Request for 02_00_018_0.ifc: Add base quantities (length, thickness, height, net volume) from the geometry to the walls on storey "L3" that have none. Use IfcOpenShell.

First a look at what the model holds.

```python
import ifcopenshell
import ifcopenshell.util.element
import ifcopenshell.util.unit

model = ifcopenshell.open("02_00_018_0.ifc")
print(model.schema)
for unit_type in ("LENGTHUNIT", "AREAUNIT", "VOLUMEUNIT"):
    print(unit_type, ifcopenshell.util.unit.calculate_unit_scale(model, unit_type))
storey = next(s for s in model.by_type("IfcBuildingStorey") if s.Name == "L3")
walls = [e for e in ifcopenshell.util.element.get_decomposition(storey) if e.is_a("IfcWall")]
for e in sorted(walls, key=lambda e: e.id()):
    print(e.id(), e.is_a(), e.Name, list(ifcopenshell.util.element.get_psets(e, qtos_only=True)), sep=" | ")
```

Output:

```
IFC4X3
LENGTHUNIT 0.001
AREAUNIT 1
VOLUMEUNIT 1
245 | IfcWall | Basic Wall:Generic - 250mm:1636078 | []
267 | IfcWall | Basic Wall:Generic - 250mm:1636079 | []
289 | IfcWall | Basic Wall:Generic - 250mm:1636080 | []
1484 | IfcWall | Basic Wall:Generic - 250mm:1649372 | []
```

```python
import ifcopenshell
import ifcopenshell.api.pset
import ifcopenshell.geom
import ifcopenshell.util.element
import ifcopenshell.util.shape
import ifcopenshell.util.unit

model = ifcopenshell.open("02_00_018_0.ifc")
unit_scale = ifcopenshell.util.unit.calculate_unit_scale(model)
volume_scale = ifcopenshell.util.unit.calculate_unit_scale(model, "VOLUMEUNIT")
settings = ifcopenshell.geom.settings()

storey = next(s for s in model.by_type("IfcBuildingStorey") if s.Name == "L3")
walls = [e for e in ifcopenshell.util.element.get_decomposition(storey) if e.is_a("IfcWall")]

for e in sorted(walls, key=lambda e: e.id()):
    if ifcopenshell.util.element.get_psets(e, qtos_only=True, should_inherit=False):
        continue
    # Geometry comes back in metres, in the element's own axes.
    shape = ifcopenshell.geom.create_shape(settings, e)
    values = {
        "Length": ifcopenshell.util.shape.get_x(shape.geometry) / unit_scale,
        "Width": ifcopenshell.util.shape.get_y(shape.geometry) / unit_scale,
        "Height": ifcopenshell.util.shape.get_z(shape.geometry) / unit_scale,
        "NetVolume": ifcopenshell.util.shape.get_volume(shape.geometry) / volume_scale,
    }
    qto = ifcopenshell.api.pset.add_qto(model, product=e, name="Qto_WallBaseQuantities")
    ifcopenshell.api.pset.edit_qto(model, qto=qto, properties=values)
    print(e.id(), {k: round(v, 3) for k, v in values.items()})

model.write("02_00_018_0_v2.ifc")
```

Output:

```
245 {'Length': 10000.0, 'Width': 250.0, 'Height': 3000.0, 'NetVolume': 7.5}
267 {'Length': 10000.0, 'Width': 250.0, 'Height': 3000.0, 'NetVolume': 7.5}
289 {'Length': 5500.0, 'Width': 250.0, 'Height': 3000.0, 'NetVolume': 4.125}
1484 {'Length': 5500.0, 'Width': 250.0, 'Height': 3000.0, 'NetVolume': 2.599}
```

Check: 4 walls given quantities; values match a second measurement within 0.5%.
